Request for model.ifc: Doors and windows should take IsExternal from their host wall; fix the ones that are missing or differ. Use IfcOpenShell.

First a look at what the model holds.

```python
import ifcopenshell
import ifcopenshell.util.element

model = ifcopenshell.open("model.ifc")
print(model.schema)
seen = {}
for e in model.by_type("IfcDoor") + model.by_type("IfcWindow"):
    if not e.FillsVoids:
        continue
    host = e.FillsVoids[0].RelatingOpeningElement.VoidsElements[0].RelatingBuildingElement
    own = ifcopenshell.util.element.get_pset(e, f"Pset_{e.is_a()[3:].removesuffix('StandardCase')}Common", "IsExternal")
    wall = ifcopenshell.util.element.get_pset(host, "Pset_WallCommon", "IsExternal")
    seen[e.is_a(), own, wall] = seen.get((e.is_a(), own, wall), 0) + 1
for (cls, own, wall), count in sorted(seen.items(), key=str):
    print(count, cls, "IsExternal:", own, "| host wall:", wall)
```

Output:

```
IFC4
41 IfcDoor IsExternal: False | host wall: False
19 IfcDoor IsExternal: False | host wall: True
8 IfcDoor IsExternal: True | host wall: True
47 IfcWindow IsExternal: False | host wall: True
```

```python
import ifcopenshell
import ifcopenshell.api.pset
import ifcopenshell.util.element

model = ifcopenshell.open("model.ifc")

count = 0
for ifc_class, pset_name in (("IfcDoor", "Pset_DoorCommon"), ("IfcWindow", "Pset_WindowCommon")):
    for e in model.by_type(ifc_class):
        if not e.FillsVoids:
            continue
        host = e.FillsVoids[0].RelatingOpeningElement.VoidsElements[0].RelatingBuildingElement
        external = ifcopenshell.util.element.get_pset(host, "Pset_WallCommon", "IsExternal")
        if external is None or ifcopenshell.util.element.get_pset(e, pset_name, "IsExternal") == external:
            continue
        pset = ifcopenshell.api.pset.add_pset(model, product=e, name=pset_name)
        ifcopenshell.api.pset.edit_pset(model, pset=pset, properties={"IsExternal": external})
        count += 1

print(count, "updated")

model.write("model-out.ifc")
```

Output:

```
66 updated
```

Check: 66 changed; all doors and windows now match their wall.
